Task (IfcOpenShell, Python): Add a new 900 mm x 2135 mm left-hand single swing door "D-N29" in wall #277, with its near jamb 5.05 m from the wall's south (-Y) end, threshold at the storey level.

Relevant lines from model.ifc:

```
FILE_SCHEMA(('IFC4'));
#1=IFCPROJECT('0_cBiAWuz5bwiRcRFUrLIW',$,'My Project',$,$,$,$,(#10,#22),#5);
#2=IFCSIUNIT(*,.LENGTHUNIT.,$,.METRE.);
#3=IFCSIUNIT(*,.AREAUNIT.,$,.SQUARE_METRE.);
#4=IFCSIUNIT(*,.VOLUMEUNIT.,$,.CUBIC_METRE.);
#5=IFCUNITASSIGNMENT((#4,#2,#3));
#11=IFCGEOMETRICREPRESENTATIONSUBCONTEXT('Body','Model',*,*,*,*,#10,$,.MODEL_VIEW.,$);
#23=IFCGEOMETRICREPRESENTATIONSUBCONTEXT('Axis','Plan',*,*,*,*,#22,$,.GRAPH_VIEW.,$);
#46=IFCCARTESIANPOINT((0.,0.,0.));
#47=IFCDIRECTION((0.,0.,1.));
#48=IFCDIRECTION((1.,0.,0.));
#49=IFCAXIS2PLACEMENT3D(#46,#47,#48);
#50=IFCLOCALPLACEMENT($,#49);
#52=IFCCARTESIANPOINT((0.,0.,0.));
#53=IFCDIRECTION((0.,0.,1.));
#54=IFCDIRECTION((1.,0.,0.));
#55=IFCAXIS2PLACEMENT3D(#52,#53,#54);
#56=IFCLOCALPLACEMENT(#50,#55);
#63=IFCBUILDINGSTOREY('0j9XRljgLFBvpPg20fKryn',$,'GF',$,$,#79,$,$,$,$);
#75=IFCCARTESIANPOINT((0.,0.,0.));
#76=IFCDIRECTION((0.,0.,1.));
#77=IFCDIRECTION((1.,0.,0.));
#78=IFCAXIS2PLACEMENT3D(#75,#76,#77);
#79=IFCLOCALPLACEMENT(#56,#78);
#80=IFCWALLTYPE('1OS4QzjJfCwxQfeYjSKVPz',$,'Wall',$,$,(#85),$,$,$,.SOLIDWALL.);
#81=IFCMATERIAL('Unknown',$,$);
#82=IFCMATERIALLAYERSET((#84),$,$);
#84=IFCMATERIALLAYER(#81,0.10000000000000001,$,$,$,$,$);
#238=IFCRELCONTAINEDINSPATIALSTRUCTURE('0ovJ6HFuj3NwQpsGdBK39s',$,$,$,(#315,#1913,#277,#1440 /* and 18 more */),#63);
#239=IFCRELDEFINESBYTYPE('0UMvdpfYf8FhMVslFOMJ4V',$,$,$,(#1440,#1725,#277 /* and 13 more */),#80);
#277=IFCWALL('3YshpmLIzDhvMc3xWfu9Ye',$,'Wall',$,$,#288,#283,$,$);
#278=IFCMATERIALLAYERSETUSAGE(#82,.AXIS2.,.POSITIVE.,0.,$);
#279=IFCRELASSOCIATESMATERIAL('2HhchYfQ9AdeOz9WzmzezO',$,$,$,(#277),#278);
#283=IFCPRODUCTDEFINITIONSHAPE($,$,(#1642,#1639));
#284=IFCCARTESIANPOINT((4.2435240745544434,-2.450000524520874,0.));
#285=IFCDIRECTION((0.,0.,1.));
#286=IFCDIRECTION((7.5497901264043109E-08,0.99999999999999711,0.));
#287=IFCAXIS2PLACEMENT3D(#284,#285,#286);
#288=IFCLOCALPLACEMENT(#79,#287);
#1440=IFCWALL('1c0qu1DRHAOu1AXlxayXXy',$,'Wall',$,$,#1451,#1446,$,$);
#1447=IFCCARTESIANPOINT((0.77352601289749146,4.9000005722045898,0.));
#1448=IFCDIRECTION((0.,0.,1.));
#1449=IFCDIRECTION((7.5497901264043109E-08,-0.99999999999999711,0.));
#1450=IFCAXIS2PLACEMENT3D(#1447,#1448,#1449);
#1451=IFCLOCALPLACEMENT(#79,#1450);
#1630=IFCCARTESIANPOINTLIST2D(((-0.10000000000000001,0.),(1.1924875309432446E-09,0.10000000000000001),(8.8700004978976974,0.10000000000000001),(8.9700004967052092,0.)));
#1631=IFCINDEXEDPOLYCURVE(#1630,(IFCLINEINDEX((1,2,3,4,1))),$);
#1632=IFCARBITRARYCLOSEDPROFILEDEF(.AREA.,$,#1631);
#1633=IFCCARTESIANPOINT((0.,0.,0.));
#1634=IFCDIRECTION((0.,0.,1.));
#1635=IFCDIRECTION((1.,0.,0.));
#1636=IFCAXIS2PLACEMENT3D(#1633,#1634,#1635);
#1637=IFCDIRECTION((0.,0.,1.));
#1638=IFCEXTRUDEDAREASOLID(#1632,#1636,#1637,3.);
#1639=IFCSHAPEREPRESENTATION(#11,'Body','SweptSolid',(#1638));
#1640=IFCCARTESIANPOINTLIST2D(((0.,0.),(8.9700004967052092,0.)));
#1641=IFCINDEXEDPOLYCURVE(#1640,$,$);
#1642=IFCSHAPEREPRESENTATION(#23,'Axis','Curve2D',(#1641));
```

```python
import numpy as np
import ifcopenshell
import ifcopenshell.api.feature
import ifcopenshell.api.geometry
import ifcopenshell.api.root
import ifcopenshell.api.spatial
import ifcopenshell.geom
import ifcopenshell.util.element
import ifcopenshell.util.placement
import ifcopenshell.util.representation
import ifcopenshell.util.shape
import ifcopenshell.util.unit

model = ifcopenshell.open("model.ifc")
unit_scale = ifcopenshell.util.unit.calculate_unit_scale(model)
settings = ifcopenshell.geom.settings()


def volume(element):
    """Net volume in cubic metres, openings subtracted."""
    shape = ifcopenshell.geom.create_shape(settings, element)
    return ifcopenshell.util.shape.get_volume(shape.geometry)


wall = model.by_id(277)
storey = ifcopenshell.util.element.get_container(wall, ifc_class="IfcBuildingStorey")
context = ifcopenshell.util.representation.get_context(model, "Model", "Body", "MODEL_VIEW")
before = volume(wall)

width, height, from_end, sill = 0.9, 2.135, 5.05, 0.0  # metres

# The wall runs along its own X axis, and the end named is its -X end.
wall_shape = ifcopenshell.geom.create_shape(settings, wall)
x, y, z = ifcopenshell.util.shape.get_vertices(wall_shape.geometry).T
start = x.min() + from_end
face, thickness = float(y.min()), float(y.max() - y.min())
wall_matrix = ifcopenshell.util.placement.get_local_placement(wall.ObjectPlacement)
level = ifcopenshell.util.placement.get_local_placement(storey.ObjectPlacement)[2, 3]


def in_wall(x, y):
    """Placement at x, y metres in the wall's axes, at sill height."""
    matrix = wall_matrix.copy()
    matrix[:, 3] = wall_matrix @ np.array([x / unit_scale, y / unit_scale, 0.0, 1.0])
    matrix[2, 3] = level + sill / unit_scale
    return matrix


# Opening: a box that overshoots both wall faces by 50 mm.
opening = ifcopenshell.api.root.create_entity(model, ifc_class="IfcOpeningElement", predefined_type="OPENING")
box = ifcopenshell.api.geometry.add_wall_representation(
    model, context=context, length=width, height=height, thickness=thickness + 0.1
)
ifcopenshell.api.geometry.assign_representation(model, product=opening, representation=box)
ifcopenshell.api.geometry.edit_object_placement(model, product=opening, matrix=in_wall(start, face - 0.05), is_si=False)
ifcopenshell.api.feature.add_feature(model, feature=opening, element=wall)

door = ifcopenshell.api.root.create_entity(model, ifc_class="IfcDoor", name="D-N29", predefined_type="DOOR")
door.OverallWidth, door.OverallHeight = width / unit_scale, height / unit_scale
door.OperationType = "SINGLE_SWING_LEFT"
body = ifcopenshell.api.geometry.add_door_representation(
    model,
    context=context,
    overall_width=door.OverallWidth,
    overall_height=door.OverallHeight,
    operation_type="SINGLE_SWING_LEFT",
    lining_properties={"LiningDepth": thickness / unit_scale, "ThresholdDepth": thickness / unit_scale},
)
ifcopenshell.api.geometry.assign_representation(model, product=door, representation=body)
ifcopenshell.api.spatial.assign_container(model, products=[door], relating_structure=storey)
ifcopenshell.api.feature.add_filling(model, opening=opening, element=door)

# The lining spans the wall, so the door starts at the wall face.
ifcopenshell.api.geometry.edit_object_placement(model, product=door, matrix=in_wall(start, face), is_si=False)

after = volume(wall)

print(f"wall volume {before:.3f} -> {after:.3f} m3")

model.write("model-out.ifc")
```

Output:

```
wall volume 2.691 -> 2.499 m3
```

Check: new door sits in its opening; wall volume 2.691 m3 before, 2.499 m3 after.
